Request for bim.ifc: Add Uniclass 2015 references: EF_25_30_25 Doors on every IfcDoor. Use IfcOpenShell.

First a look at what the model holds.

```python
import ifcopenshell

model = ifcopenshell.open("bim.ifc")
print(model.schema)
print("classifications:", [c.Name for c in model.by_type("IfcClassification")])
for ifc_class in ("IfcDoor", "IfcRoof", "IfcStair", "IfcWall", "IfcWindow"):
    print(ifc_class, len(model.by_type(ifc_class)))
```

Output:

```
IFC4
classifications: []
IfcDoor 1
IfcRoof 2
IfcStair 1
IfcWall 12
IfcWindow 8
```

```python
import ifcopenshell
import ifcopenshell.api.classification

model = ifcopenshell.open("bim.ifc")

system = ifcopenshell.api.classification.add_classification(model, classification="Uniclass 2015")

codes = {
    "IfcDoor": ("EF_25_30_25", "Doors"),
}
for ifc_class, (code, name) in codes.items():
    products = model.by_type(ifc_class)
    ifcopenshell.api.classification.add_reference(
        model, products=products, classification=system, identification=code, name=name
    )
    print(code, len(products))

model.write("bim-out.ifc")
```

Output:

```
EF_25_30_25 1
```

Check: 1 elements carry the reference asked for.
